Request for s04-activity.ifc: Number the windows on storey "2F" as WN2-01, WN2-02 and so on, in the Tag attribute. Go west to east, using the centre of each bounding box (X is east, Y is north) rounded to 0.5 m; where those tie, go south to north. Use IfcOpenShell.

First a look at what the model holds.

```python
import ifcopenshell
import ifcopenshell.util.element
import ifcopenshell.util.placement

model = ifcopenshell.open("s04-activity.ifc")
print(model.schema)
storey = next(s for s in model.by_type("IfcBuildingStorey") if s.Name == "2F")
windows = [e for e in ifcopenshell.util.element.get_decomposition(storey) if e.is_a("IfcWindow")]
for e in sorted(windows, key=lambda e: e.id()):
    origin = ifcopenshell.util.placement.get_local_placement(e.ObjectPlacement)[:3, 3]
    print(e.id(), e.Tag, e.Name, origin.round(2) + 0.0, sep=" | ")
```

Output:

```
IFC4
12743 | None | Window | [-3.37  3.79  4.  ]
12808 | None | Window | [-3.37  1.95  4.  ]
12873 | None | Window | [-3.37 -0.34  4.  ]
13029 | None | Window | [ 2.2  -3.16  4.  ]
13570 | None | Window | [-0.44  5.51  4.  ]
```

```python
import ifcopenshell
import ifcopenshell.geom
import ifcopenshell.util.element
import ifcopenshell.util.shape

model = ifcopenshell.open("s04-activity.ifc")
settings = ifcopenshell.geom.settings()
settings.set("use-world-coords", True)


def centre(element):
    shape = ifcopenshell.geom.create_shape(settings, element)
    return ifcopenshell.util.shape.get_bbox_centroid(shape.geometry)


storey = next(s for s in model.by_type("IfcBuildingStorey") if s.Name == "2F")
windows = [e for e in ifcopenshell.util.element.get_decomposition(storey) if e.is_a("IfcWindow")]

# Insertion points can sit at a corner or the storey origin, so sort by the geometry (in metres).
centres = {e: centre(e) for e in windows}
windows.sort(key=lambda e: (round(centres[e][0] / 0.5), centres[e][1]))

for i, e in enumerate(windows, start=1):
    number = f"WN2-{i:02d}"
    e.Tag = number
    print(e.id(), number)

model.write("s04-activity-out.ifc")
```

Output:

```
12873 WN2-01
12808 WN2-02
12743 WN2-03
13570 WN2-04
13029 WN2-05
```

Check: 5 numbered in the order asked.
